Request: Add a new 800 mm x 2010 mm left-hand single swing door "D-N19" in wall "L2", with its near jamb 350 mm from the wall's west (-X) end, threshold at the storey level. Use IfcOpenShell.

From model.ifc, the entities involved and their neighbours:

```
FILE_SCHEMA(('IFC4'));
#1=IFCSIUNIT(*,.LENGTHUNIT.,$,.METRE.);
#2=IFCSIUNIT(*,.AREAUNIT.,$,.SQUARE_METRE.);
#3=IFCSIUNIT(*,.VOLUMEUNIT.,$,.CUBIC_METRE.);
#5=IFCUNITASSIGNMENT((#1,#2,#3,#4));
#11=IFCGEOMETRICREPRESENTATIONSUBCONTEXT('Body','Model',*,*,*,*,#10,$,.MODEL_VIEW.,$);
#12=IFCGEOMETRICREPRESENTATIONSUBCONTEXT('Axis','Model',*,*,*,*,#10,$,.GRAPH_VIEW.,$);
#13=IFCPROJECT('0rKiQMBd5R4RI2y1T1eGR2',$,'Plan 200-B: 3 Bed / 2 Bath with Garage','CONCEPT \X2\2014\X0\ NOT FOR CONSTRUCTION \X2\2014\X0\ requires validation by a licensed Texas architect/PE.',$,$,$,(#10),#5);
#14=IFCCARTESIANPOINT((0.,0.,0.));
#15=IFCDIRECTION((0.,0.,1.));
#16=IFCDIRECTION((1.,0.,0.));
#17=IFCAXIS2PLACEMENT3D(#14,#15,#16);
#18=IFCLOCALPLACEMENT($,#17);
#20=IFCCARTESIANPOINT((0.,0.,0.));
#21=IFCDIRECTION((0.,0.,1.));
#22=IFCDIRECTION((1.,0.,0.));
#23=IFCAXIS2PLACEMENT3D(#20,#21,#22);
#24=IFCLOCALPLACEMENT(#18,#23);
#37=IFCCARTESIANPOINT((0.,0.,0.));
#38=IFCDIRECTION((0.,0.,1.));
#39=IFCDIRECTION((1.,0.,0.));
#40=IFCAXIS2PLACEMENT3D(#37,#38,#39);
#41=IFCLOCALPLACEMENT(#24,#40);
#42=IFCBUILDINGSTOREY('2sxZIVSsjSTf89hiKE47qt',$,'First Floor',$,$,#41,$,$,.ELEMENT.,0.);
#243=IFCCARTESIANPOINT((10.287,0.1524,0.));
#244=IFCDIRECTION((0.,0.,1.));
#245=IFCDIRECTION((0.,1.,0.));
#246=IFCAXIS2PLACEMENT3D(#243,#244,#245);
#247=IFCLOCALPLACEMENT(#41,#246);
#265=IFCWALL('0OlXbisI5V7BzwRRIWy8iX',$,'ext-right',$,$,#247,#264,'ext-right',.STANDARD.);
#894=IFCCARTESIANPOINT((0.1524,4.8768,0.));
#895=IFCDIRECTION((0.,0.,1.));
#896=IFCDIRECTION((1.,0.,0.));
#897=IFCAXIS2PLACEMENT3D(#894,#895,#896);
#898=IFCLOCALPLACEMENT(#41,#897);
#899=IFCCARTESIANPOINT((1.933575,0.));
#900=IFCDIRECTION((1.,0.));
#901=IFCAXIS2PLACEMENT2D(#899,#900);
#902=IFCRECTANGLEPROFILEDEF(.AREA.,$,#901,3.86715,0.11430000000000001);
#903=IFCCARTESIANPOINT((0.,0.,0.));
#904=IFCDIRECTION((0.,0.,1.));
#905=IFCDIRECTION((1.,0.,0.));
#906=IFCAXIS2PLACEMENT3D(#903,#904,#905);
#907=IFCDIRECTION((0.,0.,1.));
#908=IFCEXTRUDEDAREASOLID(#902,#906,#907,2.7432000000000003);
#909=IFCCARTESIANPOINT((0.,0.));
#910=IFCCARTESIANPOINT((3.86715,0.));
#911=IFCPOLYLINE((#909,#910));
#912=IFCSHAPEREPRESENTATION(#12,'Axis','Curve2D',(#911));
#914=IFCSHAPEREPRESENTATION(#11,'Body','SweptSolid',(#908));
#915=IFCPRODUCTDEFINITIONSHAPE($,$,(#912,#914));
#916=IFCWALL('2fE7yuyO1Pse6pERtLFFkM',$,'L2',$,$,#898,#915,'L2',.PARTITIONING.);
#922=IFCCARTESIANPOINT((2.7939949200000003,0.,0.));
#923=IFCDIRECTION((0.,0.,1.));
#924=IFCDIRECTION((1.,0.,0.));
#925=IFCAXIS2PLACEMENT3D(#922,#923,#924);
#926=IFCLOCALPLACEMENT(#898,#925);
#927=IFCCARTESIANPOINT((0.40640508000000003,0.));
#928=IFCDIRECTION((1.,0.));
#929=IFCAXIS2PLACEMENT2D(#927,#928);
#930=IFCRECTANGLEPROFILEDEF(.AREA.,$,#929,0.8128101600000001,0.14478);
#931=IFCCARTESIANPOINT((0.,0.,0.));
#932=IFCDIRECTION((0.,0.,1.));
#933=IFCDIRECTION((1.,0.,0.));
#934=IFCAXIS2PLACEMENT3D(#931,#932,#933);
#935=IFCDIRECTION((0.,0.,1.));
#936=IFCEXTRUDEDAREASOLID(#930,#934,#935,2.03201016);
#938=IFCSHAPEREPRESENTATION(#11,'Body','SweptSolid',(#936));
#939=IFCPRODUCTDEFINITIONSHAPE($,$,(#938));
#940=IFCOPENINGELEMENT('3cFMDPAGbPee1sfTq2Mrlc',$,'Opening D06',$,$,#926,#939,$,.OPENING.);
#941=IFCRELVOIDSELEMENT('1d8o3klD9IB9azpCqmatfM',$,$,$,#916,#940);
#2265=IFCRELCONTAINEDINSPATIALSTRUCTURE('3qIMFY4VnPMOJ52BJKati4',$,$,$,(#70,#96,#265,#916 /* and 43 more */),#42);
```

```python
import numpy as np
import ifcopenshell
import ifcopenshell.api.feature
import ifcopenshell.api.geometry
import ifcopenshell.api.root
import ifcopenshell.api.spatial
import ifcopenshell.geom
import ifcopenshell.util.element
import ifcopenshell.util.placement
import ifcopenshell.util.representation
import ifcopenshell.util.shape
import ifcopenshell.util.unit

model = ifcopenshell.open("model.ifc")
unit_scale = ifcopenshell.util.unit.calculate_unit_scale(model)
settings = ifcopenshell.geom.settings()


def volume(element):
    """Net volume in cubic metres, openings subtracted."""
    shape = ifcopenshell.geom.create_shape(settings, element)
    return ifcopenshell.util.shape.get_volume(shape.geometry)


wall = model.by_guid("2fE7yuyO1Pse6pERtLFFkM")
storey = ifcopenshell.util.element.get_container(wall, ifc_class="IfcBuildingStorey")
context = ifcopenshell.util.representation.get_context(model, "Model", "Body", "MODEL_VIEW")
before = volume(wall)

width, height, from_end, sill = 0.8, 2.01, 0.35, 0.0  # metres

# The wall runs along its own X axis, and the end named is its -X end.
wall_shape = ifcopenshell.geom.create_shape(settings, wall)
x, y, z = ifcopenshell.util.shape.get_vertices(wall_shape.geometry).T
start = x.min() + from_end
face, thickness = float(y.min()), float(y.max() - y.min())
wall_matrix = ifcopenshell.util.placement.get_local_placement(wall.ObjectPlacement)
level = ifcopenshell.util.placement.get_local_placement(storey.ObjectPlacement)[2, 3]


def in_wall(x, y):
    """Placement at x, y metres in the wall's axes, at sill height."""
    matrix = wall_matrix.copy()
    matrix[:, 3] = wall_matrix @ np.array([x / unit_scale, y / unit_scale, 0.0, 1.0])
    matrix[2, 3] = level + sill / unit_scale
    return matrix


# Opening: a box that overshoots both wall faces by 50 mm.
opening = ifcopenshell.api.root.create_entity(model, ifc_class="IfcOpeningElement", predefined_type="OPENING")
box = ifcopenshell.api.geometry.add_wall_representation(
    model, context=context, length=width, height=height, thickness=thickness + 0.1
)
ifcopenshell.api.geometry.assign_representation(model, product=opening, representation=box)
ifcopenshell.api.geometry.edit_object_placement(model, product=opening, matrix=in_wall(start, face - 0.05), is_si=False)
ifcopenshell.api.feature.add_feature(model, feature=opening, element=wall)

door = ifcopenshell.api.root.create_entity(model, ifc_class="IfcDoor", name="D-N19", predefined_type="DOOR")
door.OverallWidth, door.OverallHeight = width / unit_scale, height / unit_scale
door.OperationType = "SINGLE_SWING_LEFT"
body = ifcopenshell.api.geometry.add_door_representation(
    model,
    context=context,
    overall_width=door.OverallWidth,
    overall_height=door.OverallHeight,
    operation_type="SINGLE_SWING_LEFT",
    lining_properties={"LiningDepth": thickness / unit_scale, "ThresholdDepth": thickness / unit_scale},
)
ifcopenshell.api.geometry.assign_representation(model, product=door, representation=body)
ifcopenshell.api.spatial.assign_container(model, products=[door], relating_structure=storey)
ifcopenshell.api.feature.add_filling(model, opening=opening, element=door)

# The lining spans the wall, so the door starts at the wall face.
ifcopenshell.api.geometry.edit_object_placement(model, product=door, matrix=in_wall(start, face), is_si=False)

after = volume(wall)

print(f"wall volume {before:.3f} -> {after:.3f} m3")

model.write("model_updated.ifc")
```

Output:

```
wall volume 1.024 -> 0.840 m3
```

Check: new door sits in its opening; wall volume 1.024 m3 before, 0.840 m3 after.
